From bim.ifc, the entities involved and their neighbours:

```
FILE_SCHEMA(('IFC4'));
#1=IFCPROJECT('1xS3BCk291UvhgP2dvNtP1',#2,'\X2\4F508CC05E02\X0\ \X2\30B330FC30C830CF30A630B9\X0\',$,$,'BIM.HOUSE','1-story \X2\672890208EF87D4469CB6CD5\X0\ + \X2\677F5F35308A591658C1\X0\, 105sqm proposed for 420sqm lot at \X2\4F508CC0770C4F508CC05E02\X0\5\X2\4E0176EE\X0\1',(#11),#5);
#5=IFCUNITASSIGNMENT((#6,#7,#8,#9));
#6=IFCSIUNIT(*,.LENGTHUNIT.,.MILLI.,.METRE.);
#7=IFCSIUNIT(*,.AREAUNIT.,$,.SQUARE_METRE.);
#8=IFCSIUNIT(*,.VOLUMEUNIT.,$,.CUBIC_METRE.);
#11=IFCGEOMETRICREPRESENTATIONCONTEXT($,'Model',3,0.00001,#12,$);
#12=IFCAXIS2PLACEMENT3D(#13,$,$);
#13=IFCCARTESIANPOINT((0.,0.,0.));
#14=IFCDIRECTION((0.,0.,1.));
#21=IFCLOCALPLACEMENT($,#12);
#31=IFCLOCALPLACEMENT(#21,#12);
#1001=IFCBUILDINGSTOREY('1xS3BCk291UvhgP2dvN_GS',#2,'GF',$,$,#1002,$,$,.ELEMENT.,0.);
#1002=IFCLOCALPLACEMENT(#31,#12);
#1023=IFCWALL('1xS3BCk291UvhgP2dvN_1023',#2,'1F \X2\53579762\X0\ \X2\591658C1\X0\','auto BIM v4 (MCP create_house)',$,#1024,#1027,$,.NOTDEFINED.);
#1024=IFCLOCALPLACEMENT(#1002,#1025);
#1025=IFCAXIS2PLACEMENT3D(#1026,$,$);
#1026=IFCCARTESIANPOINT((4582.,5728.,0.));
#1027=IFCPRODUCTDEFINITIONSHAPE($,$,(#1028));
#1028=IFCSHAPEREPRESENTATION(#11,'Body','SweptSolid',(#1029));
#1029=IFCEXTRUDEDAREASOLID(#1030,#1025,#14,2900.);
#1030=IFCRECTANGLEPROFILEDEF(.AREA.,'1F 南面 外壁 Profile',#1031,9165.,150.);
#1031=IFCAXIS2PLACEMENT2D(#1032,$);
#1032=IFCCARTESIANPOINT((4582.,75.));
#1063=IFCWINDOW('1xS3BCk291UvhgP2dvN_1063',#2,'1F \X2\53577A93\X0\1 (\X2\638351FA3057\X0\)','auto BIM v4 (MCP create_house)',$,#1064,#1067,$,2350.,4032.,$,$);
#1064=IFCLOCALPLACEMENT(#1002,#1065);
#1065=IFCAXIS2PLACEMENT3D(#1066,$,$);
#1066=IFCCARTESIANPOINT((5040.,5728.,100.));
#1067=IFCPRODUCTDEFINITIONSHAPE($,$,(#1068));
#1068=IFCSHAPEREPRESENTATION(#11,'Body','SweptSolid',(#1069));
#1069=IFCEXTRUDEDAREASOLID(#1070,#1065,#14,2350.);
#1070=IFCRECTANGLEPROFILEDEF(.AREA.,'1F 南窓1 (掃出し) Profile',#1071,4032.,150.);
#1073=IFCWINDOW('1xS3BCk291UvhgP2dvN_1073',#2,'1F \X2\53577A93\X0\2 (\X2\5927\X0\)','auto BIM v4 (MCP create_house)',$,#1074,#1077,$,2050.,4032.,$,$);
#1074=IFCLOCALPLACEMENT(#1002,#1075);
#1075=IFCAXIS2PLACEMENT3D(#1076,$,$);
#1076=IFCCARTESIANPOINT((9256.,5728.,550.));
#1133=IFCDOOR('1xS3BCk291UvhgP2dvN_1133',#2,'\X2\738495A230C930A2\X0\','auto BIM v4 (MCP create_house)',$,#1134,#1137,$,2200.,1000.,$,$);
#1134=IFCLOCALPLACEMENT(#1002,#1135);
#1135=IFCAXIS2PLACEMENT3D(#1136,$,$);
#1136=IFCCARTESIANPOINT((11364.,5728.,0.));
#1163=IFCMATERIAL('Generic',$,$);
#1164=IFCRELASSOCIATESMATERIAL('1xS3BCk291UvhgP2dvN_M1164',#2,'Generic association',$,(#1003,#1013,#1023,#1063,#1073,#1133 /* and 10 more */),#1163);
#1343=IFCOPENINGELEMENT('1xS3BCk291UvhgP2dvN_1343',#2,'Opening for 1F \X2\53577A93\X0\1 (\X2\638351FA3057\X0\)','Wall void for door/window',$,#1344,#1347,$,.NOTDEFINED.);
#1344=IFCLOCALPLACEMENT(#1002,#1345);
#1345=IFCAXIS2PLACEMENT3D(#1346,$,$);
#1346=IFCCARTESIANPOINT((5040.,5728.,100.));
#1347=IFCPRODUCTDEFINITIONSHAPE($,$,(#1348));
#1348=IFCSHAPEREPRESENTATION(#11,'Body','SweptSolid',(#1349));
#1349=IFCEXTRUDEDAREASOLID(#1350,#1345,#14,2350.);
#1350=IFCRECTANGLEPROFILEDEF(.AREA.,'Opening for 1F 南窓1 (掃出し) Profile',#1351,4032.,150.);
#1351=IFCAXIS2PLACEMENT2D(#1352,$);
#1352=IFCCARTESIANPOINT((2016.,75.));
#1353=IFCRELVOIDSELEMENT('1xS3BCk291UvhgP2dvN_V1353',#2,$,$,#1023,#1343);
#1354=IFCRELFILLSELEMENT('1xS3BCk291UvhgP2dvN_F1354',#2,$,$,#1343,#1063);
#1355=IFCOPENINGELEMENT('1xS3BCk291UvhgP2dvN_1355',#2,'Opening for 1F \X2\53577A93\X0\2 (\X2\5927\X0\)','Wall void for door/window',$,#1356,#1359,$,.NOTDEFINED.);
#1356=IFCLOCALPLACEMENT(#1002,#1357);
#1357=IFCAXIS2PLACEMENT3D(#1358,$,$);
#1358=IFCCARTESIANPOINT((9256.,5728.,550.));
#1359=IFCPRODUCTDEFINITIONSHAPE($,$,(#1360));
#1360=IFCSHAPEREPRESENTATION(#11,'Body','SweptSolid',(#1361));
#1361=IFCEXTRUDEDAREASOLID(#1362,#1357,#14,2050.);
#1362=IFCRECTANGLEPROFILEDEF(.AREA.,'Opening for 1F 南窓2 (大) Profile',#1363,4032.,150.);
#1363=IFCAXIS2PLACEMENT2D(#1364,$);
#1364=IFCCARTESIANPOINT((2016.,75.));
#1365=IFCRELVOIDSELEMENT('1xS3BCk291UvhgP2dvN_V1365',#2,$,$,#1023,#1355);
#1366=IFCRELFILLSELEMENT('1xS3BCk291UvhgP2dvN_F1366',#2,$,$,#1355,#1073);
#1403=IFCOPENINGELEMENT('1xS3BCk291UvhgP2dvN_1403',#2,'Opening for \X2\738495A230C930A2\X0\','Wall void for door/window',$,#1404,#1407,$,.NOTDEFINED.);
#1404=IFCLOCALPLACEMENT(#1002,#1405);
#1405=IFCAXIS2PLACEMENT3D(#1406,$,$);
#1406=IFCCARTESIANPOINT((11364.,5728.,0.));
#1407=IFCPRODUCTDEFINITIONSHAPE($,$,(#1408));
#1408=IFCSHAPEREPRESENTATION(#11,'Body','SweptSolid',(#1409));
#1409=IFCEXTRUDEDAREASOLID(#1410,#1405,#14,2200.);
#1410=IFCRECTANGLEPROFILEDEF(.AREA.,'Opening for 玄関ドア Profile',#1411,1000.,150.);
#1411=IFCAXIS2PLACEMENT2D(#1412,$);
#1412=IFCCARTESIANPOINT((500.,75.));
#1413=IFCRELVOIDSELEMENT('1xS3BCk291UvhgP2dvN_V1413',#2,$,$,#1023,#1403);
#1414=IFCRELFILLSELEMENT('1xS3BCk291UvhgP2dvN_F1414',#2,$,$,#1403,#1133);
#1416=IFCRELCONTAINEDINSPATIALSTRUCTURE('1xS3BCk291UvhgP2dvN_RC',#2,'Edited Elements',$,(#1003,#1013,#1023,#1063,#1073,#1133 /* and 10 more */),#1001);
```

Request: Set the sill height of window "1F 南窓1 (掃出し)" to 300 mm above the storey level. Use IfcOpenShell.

```python
import numpy as np
import ifcopenshell
import ifcopenshell.api.geometry
import ifcopenshell.geom
import ifcopenshell.util.element
import ifcopenshell.util.placement
import ifcopenshell.util.shape
import ifcopenshell.util.unit

model = ifcopenshell.open("bim.ifc")
unit_scale = ifcopenshell.util.unit.calculate_unit_scale(model)

window = model.by_id(1063)
opening = window.FillsVoids[0].RelatingOpeningElement
storey = ifcopenshell.util.element.get_container(window, ifc_class="IfcBuildingStorey")
level = ifcopenshell.util.placement.get_local_placement(storey.ObjectPlacement)[2, 3]

# The opening's origin need not be at the sill, so measure its lowest point.
shape = ifcopenshell.geom.create_shape(ifcopenshell.geom.settings(), opening)
bottom = ifcopenshell.util.shape.get_shape_bottom_elevation(shape, shape.geometry) / unit_scale
dz = level + 0.3 / unit_scale - bottom

shift = np.array([0.0, 0.0, dz])
# The window is not placed relative to its opening, so move both.
for product in (opening, window):
    matrix = ifcopenshell.util.placement.get_local_placement(product.ObjectPlacement)
    matrix[:3, 3] += shift
    ifcopenshell.api.geometry.edit_object_placement(model, product=product, matrix=matrix, is_si=False)

print(f"moved by {dz * unit_scale:+.3f} m")

model.write("bim_v2.ifc")
```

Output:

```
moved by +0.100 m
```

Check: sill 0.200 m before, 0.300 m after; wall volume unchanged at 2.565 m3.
